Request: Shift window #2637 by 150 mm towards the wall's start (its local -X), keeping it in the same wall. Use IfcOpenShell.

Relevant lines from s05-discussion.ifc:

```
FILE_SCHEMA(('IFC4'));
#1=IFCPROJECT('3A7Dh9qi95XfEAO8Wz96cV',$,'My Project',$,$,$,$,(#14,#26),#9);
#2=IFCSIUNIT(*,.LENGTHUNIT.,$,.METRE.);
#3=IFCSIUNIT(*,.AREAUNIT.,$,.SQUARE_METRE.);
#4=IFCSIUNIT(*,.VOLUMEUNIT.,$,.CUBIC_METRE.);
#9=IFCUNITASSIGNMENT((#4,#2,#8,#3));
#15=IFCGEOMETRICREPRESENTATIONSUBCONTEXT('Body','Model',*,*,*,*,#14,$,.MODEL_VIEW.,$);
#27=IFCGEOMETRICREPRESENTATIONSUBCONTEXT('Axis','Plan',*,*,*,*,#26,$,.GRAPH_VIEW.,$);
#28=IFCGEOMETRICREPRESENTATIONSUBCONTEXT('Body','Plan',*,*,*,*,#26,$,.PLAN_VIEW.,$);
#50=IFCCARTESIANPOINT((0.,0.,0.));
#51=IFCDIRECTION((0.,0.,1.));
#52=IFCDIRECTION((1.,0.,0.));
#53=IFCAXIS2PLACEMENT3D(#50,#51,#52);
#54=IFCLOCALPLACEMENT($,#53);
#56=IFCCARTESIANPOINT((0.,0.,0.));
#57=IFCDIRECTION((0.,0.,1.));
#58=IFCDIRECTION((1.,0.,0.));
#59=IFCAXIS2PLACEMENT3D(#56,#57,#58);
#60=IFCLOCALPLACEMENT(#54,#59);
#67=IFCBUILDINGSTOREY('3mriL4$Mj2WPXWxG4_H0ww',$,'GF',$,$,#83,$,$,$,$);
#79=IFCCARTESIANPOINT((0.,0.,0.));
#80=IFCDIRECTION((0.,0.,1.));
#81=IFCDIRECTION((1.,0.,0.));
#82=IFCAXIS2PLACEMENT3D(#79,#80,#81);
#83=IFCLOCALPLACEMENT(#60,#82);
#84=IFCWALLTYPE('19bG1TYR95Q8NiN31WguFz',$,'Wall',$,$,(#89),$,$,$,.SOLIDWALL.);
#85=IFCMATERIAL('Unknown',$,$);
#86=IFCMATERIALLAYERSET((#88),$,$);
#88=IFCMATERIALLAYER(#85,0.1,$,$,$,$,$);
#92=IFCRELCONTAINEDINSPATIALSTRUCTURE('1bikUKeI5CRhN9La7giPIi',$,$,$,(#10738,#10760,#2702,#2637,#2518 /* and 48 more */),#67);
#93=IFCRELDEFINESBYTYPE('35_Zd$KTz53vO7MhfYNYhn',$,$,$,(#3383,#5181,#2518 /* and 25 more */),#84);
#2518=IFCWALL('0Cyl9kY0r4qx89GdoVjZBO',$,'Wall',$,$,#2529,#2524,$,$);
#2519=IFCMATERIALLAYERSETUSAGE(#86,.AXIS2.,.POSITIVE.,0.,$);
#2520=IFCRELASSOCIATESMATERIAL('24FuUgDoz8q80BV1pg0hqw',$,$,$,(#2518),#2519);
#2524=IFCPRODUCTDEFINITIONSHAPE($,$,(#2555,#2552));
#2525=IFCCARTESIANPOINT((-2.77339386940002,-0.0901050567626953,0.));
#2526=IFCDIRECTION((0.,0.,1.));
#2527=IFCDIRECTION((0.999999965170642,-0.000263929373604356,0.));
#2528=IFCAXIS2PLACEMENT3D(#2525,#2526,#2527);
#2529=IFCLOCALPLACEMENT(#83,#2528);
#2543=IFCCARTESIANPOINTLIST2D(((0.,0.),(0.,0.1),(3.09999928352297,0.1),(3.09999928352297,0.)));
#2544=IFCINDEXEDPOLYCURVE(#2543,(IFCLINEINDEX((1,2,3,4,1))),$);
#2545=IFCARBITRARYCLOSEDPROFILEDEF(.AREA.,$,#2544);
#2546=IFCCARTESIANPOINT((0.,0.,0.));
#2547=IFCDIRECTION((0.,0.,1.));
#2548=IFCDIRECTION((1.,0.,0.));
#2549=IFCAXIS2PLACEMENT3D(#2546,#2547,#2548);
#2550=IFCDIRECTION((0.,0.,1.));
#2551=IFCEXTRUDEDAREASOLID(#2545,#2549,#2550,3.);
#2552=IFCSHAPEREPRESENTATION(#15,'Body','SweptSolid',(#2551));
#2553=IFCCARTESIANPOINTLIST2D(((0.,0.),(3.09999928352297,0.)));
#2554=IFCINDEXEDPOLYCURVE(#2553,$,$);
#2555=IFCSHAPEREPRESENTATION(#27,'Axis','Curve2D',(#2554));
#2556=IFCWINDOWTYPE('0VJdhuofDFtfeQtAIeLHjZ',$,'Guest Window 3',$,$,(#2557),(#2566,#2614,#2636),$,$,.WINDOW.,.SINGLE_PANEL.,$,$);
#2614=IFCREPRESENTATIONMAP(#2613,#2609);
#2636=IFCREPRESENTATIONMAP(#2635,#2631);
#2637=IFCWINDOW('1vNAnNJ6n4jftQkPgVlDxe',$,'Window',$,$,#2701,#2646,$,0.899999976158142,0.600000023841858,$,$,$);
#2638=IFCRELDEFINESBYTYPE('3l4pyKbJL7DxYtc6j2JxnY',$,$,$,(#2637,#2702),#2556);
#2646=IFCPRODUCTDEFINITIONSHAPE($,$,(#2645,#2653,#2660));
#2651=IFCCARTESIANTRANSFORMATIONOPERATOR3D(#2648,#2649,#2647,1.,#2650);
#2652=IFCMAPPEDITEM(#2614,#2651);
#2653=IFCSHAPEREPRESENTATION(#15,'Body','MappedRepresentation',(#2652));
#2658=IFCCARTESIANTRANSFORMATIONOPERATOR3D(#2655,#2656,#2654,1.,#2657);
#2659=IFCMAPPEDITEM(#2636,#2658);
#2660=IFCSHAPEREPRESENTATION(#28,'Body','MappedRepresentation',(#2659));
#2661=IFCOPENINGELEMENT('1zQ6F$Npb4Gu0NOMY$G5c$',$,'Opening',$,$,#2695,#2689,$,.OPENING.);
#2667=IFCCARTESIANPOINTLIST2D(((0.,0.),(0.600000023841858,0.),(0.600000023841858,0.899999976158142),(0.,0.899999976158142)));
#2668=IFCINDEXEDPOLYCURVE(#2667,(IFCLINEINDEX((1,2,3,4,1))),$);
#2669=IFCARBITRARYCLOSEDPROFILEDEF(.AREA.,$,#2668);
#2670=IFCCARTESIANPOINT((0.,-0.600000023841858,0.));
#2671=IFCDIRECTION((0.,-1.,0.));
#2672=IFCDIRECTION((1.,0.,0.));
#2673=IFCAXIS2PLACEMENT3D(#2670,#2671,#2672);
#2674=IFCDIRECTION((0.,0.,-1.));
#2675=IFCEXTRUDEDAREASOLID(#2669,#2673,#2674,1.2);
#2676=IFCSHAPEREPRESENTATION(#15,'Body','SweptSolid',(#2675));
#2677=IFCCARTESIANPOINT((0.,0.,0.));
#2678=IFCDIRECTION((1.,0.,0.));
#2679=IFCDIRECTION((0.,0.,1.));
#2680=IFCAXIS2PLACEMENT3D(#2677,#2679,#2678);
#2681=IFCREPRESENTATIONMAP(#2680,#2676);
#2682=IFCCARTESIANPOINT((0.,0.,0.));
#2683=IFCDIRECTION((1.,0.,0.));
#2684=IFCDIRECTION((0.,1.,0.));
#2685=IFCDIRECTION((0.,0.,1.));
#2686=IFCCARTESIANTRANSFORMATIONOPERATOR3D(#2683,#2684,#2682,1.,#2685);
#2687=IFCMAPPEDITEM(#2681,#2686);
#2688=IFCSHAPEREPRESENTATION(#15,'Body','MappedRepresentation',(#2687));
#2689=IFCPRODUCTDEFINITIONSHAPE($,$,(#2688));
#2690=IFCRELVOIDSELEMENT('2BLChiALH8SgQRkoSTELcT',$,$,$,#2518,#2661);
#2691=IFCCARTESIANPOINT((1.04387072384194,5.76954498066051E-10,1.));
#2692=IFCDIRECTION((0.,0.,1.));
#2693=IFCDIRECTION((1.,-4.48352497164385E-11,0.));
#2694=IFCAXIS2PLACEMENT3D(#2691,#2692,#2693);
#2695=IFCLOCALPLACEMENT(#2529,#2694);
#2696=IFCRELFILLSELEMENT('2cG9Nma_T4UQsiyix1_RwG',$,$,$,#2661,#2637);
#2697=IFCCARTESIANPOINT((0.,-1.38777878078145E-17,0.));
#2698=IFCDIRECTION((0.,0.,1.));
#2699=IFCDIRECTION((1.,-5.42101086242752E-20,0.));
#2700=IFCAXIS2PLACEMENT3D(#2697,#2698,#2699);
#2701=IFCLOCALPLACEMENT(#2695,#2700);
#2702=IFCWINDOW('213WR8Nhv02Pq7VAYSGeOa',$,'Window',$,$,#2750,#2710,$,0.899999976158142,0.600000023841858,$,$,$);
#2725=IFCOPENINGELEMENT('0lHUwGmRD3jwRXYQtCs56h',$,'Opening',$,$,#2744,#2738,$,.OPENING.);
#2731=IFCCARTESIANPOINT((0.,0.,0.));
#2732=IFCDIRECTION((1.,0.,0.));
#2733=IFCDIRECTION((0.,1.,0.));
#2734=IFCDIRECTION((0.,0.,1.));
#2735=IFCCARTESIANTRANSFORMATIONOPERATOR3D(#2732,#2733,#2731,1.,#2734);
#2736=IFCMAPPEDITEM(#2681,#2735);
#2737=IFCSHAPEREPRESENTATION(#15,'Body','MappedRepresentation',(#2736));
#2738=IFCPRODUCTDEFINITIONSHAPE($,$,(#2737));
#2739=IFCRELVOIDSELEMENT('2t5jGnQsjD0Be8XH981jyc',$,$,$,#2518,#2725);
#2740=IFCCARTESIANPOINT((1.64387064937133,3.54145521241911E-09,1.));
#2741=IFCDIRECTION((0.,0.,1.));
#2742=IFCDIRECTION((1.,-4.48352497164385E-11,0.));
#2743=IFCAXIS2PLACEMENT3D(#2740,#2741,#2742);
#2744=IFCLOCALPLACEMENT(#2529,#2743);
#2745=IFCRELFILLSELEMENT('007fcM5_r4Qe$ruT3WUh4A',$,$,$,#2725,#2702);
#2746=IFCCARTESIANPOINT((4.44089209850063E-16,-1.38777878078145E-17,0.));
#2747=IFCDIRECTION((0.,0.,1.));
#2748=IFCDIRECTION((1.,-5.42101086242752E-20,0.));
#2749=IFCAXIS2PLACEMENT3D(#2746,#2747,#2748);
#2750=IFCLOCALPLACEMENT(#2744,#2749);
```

```python
import ifcopenshell
import ifcopenshell.api.geometry
import ifcopenshell.util.placement
import ifcopenshell.util.unit

model = ifcopenshell.open("s05-discussion.ifc")
unit_scale = ifcopenshell.util.unit.calculate_unit_scale(model)

window = model.by_id(2637)
opening = window.FillsVoids[0].RelatingOpeningElement
wall = opening.VoidsElements[0].RelatingBuildingElement

wall_matrix = ifcopenshell.util.placement.get_local_placement(wall.ObjectPlacement)
shift = wall_matrix[:3, 0] * -0.15 / unit_scale
before = ifcopenshell.util.placement.get_local_placement(window.ObjectPlacement)[:3, 3].copy()

# The window is placed relative to its opening, so it follows when the opening moves.
matrix = ifcopenshell.util.placement.get_local_placement(opening.ObjectPlacement)
matrix[:3, 3] += shift
ifcopenshell.api.geometry.edit_object_placement(
    model, product=opening, matrix=matrix, is_si=False, should_transform_children=True
)

after = ifcopenshell.util.placement.get_local_placement(window.ObjectPlacement)[:3, 3]
print("window moved by", (after - before).round(3) + 0.0)

model.write("s05-discussion_v2.ifc")
```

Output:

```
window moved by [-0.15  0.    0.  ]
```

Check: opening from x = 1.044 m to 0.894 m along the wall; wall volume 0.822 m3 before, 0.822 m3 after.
